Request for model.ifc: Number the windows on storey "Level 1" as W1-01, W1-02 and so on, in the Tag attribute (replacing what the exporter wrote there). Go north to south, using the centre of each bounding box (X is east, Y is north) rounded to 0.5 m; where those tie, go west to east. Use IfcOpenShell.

First a look at what the model holds.

```python
import ifcopenshell
import ifcopenshell.util.element
import ifcopenshell.util.placement

model = ifcopenshell.open("model.ifc")
print(model.schema)
storey = next(s for s in model.by_type("IfcBuildingStorey") if s.Name == "Level 1")
windows = [e for e in ifcopenshell.util.element.get_decomposition(storey) if e.is_a("IfcWindow")]
for e in sorted(windows, key=lambda e: e.id()):
    origin = ifcopenshell.util.placement.get_local_placement(e.ObjectPlacement)[:3, 3]
    print(e.id(), e.Tag, e.Name, origin.round(2) + 0.0, sep=" | ")
```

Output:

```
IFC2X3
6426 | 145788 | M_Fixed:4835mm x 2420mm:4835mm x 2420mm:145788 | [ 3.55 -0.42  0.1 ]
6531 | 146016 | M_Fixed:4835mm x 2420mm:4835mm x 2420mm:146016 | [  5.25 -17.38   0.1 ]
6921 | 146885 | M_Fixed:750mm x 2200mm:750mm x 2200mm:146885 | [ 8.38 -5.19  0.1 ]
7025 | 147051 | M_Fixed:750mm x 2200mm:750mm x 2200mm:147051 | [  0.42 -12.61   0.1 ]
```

```python
import ifcopenshell
import ifcopenshell.geom
import ifcopenshell.util.element
import ifcopenshell.util.shape

model = ifcopenshell.open("model.ifc")
settings = ifcopenshell.geom.settings()
settings.set("use-world-coords", True)


def centre(element):
    shape = ifcopenshell.geom.create_shape(settings, element)
    return ifcopenshell.util.shape.get_bbox_centroid(shape.geometry)


storey = next(s for s in model.by_type("IfcBuildingStorey") if s.Name == "Level 1")
windows = [e for e in ifcopenshell.util.element.get_decomposition(storey) if e.is_a("IfcWindow")]

# Insertion points can sit at a corner or the storey origin, so sort by the geometry (in metres).
centres = {e: centre(e) for e in windows}
windows.sort(key=lambda e: (-round(centres[e][1] / 0.5), centres[e][0]))

for i, e in enumerate(windows, start=1):
    number = f"W1-{i:02d}"
    e.Tag = number
    print(e.id(), number)

model.write("model_v2.ifc")
```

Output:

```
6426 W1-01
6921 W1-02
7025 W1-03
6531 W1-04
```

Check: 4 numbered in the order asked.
